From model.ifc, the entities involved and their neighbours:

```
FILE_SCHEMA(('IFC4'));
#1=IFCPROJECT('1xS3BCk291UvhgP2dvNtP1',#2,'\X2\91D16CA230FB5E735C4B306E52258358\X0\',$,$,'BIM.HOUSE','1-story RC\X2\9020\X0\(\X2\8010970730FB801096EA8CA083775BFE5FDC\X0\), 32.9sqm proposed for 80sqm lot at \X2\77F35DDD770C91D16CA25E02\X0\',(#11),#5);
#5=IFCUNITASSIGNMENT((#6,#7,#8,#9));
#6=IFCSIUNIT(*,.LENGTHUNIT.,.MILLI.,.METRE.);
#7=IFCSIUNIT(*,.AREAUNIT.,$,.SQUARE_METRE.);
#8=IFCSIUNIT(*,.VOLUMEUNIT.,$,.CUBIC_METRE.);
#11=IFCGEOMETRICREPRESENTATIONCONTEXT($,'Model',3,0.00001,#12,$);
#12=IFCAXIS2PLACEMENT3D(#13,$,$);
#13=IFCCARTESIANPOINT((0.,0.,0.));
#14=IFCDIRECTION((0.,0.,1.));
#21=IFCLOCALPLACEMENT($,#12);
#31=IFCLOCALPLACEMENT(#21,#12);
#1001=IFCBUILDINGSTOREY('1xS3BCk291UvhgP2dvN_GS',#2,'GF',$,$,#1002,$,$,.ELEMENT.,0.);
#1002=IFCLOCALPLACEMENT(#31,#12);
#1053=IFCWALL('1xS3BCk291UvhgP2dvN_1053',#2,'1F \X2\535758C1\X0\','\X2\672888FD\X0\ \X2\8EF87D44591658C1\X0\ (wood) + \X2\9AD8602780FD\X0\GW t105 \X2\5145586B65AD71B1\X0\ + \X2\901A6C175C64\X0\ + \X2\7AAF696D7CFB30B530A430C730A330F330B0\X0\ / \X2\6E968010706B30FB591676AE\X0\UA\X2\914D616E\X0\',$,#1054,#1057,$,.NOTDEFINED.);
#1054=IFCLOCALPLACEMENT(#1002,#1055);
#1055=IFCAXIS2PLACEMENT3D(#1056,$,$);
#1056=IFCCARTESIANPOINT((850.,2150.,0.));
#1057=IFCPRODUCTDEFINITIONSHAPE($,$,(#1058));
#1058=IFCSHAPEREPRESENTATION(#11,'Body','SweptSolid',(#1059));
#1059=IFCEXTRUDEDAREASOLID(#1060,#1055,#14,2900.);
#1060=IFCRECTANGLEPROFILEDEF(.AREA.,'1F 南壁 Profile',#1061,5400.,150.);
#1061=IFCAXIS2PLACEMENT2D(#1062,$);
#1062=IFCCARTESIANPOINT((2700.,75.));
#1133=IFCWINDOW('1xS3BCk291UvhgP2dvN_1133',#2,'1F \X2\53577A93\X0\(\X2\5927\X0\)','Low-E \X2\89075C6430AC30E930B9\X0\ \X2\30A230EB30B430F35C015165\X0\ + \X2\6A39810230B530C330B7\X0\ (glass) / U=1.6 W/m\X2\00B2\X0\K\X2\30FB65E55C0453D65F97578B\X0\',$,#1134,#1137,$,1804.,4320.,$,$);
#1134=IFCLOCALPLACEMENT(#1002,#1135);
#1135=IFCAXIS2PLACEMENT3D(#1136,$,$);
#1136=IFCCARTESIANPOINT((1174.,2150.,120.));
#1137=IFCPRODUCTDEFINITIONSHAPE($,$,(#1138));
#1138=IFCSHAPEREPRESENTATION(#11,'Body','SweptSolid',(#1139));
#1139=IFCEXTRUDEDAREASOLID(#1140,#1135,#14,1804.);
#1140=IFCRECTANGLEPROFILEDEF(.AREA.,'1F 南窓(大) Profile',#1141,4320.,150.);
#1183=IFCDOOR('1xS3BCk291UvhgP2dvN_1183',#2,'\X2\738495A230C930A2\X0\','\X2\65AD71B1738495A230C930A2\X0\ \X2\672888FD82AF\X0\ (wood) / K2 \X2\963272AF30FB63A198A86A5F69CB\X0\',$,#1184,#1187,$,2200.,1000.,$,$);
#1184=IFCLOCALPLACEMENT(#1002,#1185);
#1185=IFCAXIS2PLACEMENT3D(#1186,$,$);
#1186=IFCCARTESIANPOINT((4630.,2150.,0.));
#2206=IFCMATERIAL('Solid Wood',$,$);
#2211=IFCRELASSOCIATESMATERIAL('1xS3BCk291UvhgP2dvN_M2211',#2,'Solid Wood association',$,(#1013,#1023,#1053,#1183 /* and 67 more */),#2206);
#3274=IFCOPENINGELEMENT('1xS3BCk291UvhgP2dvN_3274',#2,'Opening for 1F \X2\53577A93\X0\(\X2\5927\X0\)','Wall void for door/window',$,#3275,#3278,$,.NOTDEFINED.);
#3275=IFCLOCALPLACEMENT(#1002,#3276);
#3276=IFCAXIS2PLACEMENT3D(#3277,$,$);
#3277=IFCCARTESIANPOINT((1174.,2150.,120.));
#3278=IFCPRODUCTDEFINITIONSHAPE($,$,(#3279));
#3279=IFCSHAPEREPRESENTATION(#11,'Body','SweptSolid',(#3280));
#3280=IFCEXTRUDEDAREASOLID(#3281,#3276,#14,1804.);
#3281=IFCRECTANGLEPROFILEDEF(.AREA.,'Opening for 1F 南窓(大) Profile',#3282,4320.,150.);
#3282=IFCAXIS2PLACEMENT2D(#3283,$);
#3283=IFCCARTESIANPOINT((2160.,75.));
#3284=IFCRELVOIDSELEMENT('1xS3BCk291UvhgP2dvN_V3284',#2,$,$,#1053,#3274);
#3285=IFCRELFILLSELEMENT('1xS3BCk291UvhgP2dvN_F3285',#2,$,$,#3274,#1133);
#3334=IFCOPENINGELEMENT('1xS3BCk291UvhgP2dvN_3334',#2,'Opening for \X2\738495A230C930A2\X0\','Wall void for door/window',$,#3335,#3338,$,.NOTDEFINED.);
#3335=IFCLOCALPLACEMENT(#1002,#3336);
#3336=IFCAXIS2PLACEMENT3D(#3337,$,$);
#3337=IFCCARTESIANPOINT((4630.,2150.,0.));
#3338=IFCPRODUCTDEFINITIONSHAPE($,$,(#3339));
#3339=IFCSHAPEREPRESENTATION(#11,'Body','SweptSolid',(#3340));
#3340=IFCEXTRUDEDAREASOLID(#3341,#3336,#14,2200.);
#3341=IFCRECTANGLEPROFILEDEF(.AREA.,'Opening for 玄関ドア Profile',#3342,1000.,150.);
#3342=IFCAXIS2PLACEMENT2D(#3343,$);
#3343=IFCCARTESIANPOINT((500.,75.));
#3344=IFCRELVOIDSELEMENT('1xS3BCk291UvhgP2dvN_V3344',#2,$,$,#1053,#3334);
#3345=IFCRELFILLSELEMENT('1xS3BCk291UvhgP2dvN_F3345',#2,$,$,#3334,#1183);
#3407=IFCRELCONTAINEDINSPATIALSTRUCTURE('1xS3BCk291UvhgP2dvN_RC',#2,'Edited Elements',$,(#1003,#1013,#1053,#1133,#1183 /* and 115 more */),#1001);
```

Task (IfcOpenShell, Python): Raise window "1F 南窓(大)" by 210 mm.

```python
import numpy as np
import ifcopenshell
import ifcopenshell.api.geometry
import ifcopenshell.util.placement
import ifcopenshell.util.unit

model = ifcopenshell.open("model.ifc")
unit_scale = ifcopenshell.util.unit.calculate_unit_scale(model)

window = model.by_id(1133)
opening = window.FillsVoids[0].RelatingOpeningElement
dz = 210.0

shift = np.array([0.0, 0.0, dz])
# The window is not placed relative to its opening, so move both.
for product in (opening, window):
    matrix = ifcopenshell.util.placement.get_local_placement(product.ObjectPlacement)
    matrix[:3, 3] += shift
    ifcopenshell.api.geometry.edit_object_placement(model, product=product, matrix=matrix, is_si=False)

print(f"moved by {dz * unit_scale:+.3f} m")

model.write("model_rev.ifc")
```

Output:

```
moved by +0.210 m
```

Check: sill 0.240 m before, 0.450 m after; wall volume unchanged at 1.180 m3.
